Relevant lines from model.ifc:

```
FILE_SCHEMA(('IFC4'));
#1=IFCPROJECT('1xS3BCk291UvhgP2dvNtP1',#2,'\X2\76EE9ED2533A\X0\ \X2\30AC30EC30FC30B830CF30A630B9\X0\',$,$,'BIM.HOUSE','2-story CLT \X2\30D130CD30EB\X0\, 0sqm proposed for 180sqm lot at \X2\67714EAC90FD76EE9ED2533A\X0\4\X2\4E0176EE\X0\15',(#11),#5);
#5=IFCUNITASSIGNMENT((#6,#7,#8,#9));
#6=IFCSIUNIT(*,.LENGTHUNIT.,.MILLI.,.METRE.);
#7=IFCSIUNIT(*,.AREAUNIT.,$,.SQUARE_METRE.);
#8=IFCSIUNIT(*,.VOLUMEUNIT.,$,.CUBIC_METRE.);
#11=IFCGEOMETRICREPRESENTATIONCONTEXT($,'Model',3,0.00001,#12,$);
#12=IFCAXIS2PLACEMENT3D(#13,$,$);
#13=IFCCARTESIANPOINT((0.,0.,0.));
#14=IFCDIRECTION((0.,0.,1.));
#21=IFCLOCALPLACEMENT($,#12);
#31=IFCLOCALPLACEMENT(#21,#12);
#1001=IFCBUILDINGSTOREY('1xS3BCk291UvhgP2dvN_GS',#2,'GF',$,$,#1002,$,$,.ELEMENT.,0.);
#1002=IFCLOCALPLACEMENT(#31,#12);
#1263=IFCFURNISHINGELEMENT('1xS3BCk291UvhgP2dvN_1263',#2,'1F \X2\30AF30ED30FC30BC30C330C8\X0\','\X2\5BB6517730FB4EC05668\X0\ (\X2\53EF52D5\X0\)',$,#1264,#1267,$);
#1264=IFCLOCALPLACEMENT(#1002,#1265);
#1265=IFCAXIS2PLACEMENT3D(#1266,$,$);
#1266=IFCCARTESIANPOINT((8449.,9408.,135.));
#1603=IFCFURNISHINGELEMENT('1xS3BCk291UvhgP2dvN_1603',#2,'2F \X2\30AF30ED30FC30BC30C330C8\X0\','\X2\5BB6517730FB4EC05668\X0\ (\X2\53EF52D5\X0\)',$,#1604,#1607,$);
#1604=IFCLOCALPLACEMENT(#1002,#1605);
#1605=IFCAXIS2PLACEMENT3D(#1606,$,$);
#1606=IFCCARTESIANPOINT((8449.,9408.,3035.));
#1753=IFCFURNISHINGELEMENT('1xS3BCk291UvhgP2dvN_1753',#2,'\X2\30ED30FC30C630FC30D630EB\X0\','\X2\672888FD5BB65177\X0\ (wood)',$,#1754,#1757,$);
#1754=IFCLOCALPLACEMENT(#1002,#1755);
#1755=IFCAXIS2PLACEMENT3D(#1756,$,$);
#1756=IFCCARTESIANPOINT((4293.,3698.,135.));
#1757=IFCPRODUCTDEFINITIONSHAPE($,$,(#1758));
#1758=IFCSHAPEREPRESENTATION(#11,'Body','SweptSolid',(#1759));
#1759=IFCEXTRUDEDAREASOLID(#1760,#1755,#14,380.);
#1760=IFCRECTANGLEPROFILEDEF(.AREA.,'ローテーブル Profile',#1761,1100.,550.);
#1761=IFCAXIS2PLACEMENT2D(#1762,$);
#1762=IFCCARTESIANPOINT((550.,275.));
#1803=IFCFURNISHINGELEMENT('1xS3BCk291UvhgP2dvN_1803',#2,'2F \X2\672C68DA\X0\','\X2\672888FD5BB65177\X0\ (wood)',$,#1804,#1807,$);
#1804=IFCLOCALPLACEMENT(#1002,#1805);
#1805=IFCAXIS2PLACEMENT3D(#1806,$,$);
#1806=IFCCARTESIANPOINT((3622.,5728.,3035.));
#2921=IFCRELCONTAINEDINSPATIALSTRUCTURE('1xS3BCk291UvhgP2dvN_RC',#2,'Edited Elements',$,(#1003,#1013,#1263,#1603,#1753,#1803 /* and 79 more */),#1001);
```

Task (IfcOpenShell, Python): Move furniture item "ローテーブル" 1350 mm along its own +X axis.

```python
import ifcopenshell
import ifcopenshell.api.geometry
import ifcopenshell.util.placement
import ifcopenshell.util.unit

model = ifcopenshell.open("model.ifc")
unit_scale = ifcopenshell.util.unit.calculate_unit_scale(model)

item = model.by_guid("1xS3BCk291UvhgP2dvN_1753")
matrix = ifcopenshell.util.placement.get_local_placement(item.ObjectPlacement)
matrix[:3, 3] += matrix[:3, 0] * 1.35 / unit_scale
ifcopenshell.api.geometry.edit_object_placement(model, product=item, matrix=matrix, is_si=False)

print(ifcopenshell.util.placement.get_local_placement(item.ObjectPlacement).round(3) + 0.0)

model.write("model_rev.ifc")
```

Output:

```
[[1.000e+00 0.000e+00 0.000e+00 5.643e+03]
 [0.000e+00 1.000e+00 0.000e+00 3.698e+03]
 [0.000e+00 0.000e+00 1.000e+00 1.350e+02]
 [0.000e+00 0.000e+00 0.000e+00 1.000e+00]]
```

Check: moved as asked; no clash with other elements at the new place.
